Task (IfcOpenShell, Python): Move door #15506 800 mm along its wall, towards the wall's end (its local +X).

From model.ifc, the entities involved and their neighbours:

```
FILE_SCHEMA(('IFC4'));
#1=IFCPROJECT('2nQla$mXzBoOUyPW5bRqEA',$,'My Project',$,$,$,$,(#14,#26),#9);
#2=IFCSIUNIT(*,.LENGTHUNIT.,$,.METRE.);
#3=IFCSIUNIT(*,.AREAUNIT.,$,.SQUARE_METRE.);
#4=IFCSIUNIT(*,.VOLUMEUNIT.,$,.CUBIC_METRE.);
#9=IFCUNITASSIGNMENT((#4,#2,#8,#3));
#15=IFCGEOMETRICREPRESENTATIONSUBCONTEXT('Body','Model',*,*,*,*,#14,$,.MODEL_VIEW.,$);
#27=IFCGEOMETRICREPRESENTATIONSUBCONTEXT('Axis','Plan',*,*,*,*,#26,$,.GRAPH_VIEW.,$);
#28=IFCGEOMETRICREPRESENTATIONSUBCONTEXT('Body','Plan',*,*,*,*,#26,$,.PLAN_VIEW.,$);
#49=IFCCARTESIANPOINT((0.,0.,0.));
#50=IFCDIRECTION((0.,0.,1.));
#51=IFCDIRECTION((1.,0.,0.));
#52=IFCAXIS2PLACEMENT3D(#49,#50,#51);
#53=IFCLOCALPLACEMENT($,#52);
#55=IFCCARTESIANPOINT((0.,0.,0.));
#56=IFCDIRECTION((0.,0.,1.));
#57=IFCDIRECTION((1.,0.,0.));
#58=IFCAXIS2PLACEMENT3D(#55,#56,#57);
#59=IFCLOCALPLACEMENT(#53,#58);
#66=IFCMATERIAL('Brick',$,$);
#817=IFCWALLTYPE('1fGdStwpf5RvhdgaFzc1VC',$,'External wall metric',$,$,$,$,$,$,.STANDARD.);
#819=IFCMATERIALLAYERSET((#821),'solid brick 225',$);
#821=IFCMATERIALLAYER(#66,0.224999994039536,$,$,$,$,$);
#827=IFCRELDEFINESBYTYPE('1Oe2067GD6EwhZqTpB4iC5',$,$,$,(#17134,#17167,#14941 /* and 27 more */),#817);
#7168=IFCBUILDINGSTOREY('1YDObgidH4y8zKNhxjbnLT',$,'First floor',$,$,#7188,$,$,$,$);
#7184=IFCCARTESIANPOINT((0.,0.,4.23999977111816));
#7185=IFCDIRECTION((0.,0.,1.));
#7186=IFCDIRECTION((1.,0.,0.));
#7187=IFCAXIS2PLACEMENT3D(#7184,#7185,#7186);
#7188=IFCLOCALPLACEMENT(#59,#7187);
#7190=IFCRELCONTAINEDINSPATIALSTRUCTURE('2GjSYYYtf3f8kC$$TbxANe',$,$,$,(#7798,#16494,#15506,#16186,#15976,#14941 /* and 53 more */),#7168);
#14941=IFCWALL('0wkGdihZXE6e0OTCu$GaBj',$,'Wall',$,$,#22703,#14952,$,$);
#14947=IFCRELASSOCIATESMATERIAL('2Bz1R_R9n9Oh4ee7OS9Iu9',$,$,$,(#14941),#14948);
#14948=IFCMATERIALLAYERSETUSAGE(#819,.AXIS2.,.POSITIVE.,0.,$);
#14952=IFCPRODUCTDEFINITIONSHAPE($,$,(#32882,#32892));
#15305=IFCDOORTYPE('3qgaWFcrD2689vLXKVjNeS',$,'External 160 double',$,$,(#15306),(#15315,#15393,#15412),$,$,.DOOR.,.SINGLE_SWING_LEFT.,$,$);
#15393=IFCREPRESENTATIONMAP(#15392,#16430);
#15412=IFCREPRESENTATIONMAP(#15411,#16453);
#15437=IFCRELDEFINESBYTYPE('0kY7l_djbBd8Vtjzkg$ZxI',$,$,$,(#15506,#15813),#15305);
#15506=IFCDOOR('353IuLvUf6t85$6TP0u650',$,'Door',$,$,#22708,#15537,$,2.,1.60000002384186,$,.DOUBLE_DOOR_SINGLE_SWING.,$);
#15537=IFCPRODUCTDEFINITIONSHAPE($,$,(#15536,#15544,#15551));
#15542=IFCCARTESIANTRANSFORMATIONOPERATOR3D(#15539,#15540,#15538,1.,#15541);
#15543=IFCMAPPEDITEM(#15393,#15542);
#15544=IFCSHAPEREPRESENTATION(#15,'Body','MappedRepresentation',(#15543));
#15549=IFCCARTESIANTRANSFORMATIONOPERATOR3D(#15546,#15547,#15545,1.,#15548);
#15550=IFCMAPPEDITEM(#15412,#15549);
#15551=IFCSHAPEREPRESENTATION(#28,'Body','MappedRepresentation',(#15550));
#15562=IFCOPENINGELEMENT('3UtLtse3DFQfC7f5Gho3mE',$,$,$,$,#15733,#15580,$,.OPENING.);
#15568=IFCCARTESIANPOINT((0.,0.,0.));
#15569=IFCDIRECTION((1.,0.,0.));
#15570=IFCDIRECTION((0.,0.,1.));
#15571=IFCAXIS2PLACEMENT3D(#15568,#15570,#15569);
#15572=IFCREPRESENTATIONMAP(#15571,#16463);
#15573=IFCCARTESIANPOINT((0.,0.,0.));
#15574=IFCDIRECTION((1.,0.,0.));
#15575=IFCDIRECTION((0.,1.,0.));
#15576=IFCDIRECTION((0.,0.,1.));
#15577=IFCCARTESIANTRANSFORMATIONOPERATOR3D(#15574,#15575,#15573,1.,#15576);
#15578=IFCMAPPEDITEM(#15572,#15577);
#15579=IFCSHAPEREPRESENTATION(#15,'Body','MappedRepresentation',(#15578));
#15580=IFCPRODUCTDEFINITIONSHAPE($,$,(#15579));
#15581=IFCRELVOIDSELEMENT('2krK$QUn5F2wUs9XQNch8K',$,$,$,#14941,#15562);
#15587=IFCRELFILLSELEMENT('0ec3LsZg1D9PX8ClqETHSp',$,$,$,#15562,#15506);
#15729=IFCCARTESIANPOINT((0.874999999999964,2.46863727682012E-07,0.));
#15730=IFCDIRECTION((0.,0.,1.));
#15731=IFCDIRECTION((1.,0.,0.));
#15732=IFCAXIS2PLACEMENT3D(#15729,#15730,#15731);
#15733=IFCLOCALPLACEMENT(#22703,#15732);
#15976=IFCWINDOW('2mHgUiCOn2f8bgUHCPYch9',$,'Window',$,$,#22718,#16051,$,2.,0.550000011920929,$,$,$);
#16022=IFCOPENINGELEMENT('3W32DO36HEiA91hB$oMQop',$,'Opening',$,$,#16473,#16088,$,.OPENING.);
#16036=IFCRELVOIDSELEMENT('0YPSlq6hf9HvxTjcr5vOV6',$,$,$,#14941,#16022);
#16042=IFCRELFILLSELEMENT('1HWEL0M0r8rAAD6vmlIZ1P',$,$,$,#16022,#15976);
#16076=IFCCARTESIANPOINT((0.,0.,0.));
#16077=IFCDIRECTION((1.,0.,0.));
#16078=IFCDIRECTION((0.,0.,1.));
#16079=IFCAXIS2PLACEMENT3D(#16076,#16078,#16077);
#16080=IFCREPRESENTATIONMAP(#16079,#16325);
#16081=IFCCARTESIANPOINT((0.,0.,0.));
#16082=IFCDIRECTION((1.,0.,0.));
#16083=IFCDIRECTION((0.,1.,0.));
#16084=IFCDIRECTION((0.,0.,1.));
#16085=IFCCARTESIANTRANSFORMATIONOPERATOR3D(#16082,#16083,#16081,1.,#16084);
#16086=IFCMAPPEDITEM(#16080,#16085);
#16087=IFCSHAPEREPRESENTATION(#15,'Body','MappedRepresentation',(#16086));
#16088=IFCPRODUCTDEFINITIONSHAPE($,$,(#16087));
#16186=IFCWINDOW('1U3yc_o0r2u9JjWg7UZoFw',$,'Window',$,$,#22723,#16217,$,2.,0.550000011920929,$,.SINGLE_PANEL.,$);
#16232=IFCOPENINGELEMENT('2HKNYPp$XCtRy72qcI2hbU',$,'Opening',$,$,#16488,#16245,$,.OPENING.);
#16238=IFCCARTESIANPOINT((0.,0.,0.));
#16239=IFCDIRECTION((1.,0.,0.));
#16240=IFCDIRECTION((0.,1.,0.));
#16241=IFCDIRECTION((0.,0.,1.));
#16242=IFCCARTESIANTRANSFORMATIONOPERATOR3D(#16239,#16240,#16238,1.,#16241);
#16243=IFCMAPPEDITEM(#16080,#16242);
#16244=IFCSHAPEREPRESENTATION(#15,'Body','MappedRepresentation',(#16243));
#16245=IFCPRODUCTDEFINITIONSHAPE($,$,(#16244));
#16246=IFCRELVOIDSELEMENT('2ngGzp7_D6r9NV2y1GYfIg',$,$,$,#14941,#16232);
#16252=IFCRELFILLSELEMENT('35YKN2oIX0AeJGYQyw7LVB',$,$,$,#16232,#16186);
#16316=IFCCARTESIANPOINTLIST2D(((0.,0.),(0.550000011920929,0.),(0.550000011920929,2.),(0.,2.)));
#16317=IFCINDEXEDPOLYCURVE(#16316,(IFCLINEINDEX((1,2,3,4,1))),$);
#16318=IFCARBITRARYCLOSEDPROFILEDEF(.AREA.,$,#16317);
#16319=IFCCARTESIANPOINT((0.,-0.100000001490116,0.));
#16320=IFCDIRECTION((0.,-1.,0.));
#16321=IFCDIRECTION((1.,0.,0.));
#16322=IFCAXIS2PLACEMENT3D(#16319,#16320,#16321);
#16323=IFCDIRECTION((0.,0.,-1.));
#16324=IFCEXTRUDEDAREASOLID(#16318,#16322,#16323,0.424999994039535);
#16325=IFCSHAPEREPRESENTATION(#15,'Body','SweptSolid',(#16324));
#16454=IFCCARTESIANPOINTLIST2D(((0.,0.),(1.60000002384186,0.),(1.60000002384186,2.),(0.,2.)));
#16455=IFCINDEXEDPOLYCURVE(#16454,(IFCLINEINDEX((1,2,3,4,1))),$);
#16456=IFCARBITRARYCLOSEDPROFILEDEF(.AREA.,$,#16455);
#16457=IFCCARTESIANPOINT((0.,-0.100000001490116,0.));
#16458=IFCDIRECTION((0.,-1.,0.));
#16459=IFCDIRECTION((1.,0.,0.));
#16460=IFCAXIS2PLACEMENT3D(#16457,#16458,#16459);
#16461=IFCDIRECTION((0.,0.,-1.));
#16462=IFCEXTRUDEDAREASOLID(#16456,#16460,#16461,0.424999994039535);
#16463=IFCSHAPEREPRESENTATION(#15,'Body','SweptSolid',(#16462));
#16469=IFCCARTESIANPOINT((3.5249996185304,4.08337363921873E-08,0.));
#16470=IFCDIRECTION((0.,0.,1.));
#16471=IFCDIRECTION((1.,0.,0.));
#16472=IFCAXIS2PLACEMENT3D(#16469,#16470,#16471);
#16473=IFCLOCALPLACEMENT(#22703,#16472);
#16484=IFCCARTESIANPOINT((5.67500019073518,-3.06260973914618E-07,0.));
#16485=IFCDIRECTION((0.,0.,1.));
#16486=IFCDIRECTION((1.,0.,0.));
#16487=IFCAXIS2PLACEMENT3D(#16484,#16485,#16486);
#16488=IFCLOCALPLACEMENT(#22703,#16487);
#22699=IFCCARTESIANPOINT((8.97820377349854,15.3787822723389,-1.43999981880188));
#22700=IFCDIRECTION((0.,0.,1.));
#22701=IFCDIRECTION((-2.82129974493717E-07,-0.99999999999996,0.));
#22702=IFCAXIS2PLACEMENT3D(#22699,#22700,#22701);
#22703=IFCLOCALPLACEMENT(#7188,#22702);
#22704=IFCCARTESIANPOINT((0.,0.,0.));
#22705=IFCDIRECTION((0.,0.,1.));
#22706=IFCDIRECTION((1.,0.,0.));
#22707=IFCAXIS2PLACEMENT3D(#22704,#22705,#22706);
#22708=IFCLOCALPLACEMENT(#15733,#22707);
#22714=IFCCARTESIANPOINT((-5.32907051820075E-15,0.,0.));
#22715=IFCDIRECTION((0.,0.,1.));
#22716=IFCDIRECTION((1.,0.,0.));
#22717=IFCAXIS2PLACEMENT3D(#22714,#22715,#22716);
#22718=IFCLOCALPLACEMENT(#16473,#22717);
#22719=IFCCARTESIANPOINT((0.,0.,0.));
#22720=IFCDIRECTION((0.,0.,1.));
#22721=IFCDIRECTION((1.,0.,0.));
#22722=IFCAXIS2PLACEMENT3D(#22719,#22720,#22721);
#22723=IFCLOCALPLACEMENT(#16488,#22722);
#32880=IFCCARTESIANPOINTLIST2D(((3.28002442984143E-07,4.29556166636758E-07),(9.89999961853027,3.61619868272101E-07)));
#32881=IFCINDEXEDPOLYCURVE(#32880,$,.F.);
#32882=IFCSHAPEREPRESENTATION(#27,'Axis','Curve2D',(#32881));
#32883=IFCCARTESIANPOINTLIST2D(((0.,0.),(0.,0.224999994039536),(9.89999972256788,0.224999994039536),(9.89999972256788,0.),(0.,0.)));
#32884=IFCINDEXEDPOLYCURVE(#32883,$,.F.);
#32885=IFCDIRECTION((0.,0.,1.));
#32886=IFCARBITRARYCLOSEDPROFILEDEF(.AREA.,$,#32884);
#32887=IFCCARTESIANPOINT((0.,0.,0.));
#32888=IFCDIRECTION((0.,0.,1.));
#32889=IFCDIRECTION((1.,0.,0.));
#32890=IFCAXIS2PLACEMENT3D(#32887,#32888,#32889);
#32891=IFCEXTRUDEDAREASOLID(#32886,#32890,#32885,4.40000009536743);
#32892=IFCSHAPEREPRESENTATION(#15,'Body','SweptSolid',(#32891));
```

```python
import ifcopenshell
import ifcopenshell.api.geometry
import ifcopenshell.util.placement
import ifcopenshell.util.unit

model = ifcopenshell.open("model.ifc")
unit_scale = ifcopenshell.util.unit.calculate_unit_scale(model)

door = model.by_guid("353IuLvUf6t85$6TP0u650")
opening = door.FillsVoids[0].RelatingOpeningElement
wall = opening.VoidsElements[0].RelatingBuildingElement

wall_matrix = ifcopenshell.util.placement.get_local_placement(wall.ObjectPlacement)
shift = wall_matrix[:3, 0] * 0.8 / unit_scale
before = ifcopenshell.util.placement.get_local_placement(door.ObjectPlacement)[:3, 3].copy()

# The door is placed relative to its opening, so it follows when the opening moves.
matrix = ifcopenshell.util.placement.get_local_placement(opening.ObjectPlacement)
matrix[:3, 3] += shift
ifcopenshell.api.geometry.edit_object_placement(
    model, product=opening, matrix=matrix, is_si=False, should_transform_children=True
)

after = ifcopenshell.util.placement.get_local_placement(door.ObjectPlacement)[:3, 3]
print("door moved by", (after - before).round(3) + 0.0)

model.write("model_edited.ifc")
```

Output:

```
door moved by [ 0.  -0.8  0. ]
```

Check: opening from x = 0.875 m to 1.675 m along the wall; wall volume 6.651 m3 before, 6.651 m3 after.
